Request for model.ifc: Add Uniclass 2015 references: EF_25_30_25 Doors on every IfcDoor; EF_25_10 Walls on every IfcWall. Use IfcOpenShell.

First a look at what the model holds.

```python
import ifcopenshell

model = ifcopenshell.open("model.ifc")
print(model.schema)
print("classifications:", [c.Name for c in model.by_type("IfcClassification")])
for ifc_class in ("IfcDoor", "IfcRoof", "IfcStair", "IfcWall", "IfcWindow"):
    print(ifc_class, len(model.by_type(ifc_class)))
```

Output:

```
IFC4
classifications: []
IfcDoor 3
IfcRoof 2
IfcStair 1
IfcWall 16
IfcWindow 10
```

```python
import ifcopenshell
import ifcopenshell.api.classification

model = ifcopenshell.open("model.ifc")

system = ifcopenshell.api.classification.add_classification(model, classification="Uniclass 2015")

codes = {
    "IfcDoor": ("EF_25_30_25", "Doors"),
    "IfcWall": ("EF_25_10", "Walls"),
}
for ifc_class, (code, name) in codes.items():
    products = model.by_type(ifc_class)
    ifcopenshell.api.classification.add_reference(
        model, products=products, classification=system, identification=code, name=name
    )
    print(code, len(products))

model.write("model_edited.ifc")
```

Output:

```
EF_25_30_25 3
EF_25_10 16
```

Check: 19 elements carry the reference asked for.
